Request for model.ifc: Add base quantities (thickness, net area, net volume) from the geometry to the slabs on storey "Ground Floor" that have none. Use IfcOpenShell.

First a look at what the model holds.

```python
import ifcopenshell
import ifcopenshell.util.element
import ifcopenshell.util.unit

model = ifcopenshell.open("model.ifc")
print(model.schema)
for unit_type in ("LENGTHUNIT", "AREAUNIT", "VOLUMEUNIT"):
    print(unit_type, ifcopenshell.util.unit.calculate_unit_scale(model, unit_type))
storey = next(s for s in model.by_type("IfcBuildingStorey") if s.Name == "Ground Floor")
slabs = [e for e in ifcopenshell.util.element.get_decomposition(storey) if e.is_a("IfcSlab")]
for e in sorted(slabs, key=lambda e: e.id()):
    print(e.id(), e.is_a(), e.Name, list(ifcopenshell.util.element.get_psets(e, qtos_only=True)), sep=" | ")
```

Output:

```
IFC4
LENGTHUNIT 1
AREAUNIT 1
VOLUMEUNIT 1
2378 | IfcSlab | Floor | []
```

```python
import ifcopenshell
import ifcopenshell.api.pset
import ifcopenshell.geom
import ifcopenshell.util.element
import ifcopenshell.util.shape
import ifcopenshell.util.unit

model = ifcopenshell.open("model.ifc")
unit_scale = ifcopenshell.util.unit.calculate_unit_scale(model)
area_scale = ifcopenshell.util.unit.calculate_unit_scale(model, "AREAUNIT")
volume_scale = ifcopenshell.util.unit.calculate_unit_scale(model, "VOLUMEUNIT")
settings = ifcopenshell.geom.settings()

storey = next(s for s in model.by_type("IfcBuildingStorey") if s.Name == "Ground Floor")
slabs = [e for e in ifcopenshell.util.element.get_decomposition(storey) if e.is_a("IfcSlab")]

for e in sorted(slabs, key=lambda e: e.id()):
    if ifcopenshell.util.element.get_psets(e, qtos_only=True, should_inherit=False):
        continue
    # Geometry comes back in metres, in the element's own axes.
    shape = ifcopenshell.geom.create_shape(settings, e)
    values = {
        "Width": ifcopenshell.util.shape.get_z(shape.geometry) / unit_scale,
        "NetArea": ifcopenshell.util.shape.get_footprint_area(shape.geometry) / area_scale,
        "NetVolume": ifcopenshell.util.shape.get_volume(shape.geometry) / volume_scale,
    }
    qto = ifcopenshell.api.pset.add_qto(model, product=e, name="Qto_SlabBaseQuantities")
    ifcopenshell.api.pset.edit_qto(model, qto=qto, properties=values)
    print(e.id(), {k: round(v, 3) for k, v in values.items()})

model.write("model_updated.ifc")
```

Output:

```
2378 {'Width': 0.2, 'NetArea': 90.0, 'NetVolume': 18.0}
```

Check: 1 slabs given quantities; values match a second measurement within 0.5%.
